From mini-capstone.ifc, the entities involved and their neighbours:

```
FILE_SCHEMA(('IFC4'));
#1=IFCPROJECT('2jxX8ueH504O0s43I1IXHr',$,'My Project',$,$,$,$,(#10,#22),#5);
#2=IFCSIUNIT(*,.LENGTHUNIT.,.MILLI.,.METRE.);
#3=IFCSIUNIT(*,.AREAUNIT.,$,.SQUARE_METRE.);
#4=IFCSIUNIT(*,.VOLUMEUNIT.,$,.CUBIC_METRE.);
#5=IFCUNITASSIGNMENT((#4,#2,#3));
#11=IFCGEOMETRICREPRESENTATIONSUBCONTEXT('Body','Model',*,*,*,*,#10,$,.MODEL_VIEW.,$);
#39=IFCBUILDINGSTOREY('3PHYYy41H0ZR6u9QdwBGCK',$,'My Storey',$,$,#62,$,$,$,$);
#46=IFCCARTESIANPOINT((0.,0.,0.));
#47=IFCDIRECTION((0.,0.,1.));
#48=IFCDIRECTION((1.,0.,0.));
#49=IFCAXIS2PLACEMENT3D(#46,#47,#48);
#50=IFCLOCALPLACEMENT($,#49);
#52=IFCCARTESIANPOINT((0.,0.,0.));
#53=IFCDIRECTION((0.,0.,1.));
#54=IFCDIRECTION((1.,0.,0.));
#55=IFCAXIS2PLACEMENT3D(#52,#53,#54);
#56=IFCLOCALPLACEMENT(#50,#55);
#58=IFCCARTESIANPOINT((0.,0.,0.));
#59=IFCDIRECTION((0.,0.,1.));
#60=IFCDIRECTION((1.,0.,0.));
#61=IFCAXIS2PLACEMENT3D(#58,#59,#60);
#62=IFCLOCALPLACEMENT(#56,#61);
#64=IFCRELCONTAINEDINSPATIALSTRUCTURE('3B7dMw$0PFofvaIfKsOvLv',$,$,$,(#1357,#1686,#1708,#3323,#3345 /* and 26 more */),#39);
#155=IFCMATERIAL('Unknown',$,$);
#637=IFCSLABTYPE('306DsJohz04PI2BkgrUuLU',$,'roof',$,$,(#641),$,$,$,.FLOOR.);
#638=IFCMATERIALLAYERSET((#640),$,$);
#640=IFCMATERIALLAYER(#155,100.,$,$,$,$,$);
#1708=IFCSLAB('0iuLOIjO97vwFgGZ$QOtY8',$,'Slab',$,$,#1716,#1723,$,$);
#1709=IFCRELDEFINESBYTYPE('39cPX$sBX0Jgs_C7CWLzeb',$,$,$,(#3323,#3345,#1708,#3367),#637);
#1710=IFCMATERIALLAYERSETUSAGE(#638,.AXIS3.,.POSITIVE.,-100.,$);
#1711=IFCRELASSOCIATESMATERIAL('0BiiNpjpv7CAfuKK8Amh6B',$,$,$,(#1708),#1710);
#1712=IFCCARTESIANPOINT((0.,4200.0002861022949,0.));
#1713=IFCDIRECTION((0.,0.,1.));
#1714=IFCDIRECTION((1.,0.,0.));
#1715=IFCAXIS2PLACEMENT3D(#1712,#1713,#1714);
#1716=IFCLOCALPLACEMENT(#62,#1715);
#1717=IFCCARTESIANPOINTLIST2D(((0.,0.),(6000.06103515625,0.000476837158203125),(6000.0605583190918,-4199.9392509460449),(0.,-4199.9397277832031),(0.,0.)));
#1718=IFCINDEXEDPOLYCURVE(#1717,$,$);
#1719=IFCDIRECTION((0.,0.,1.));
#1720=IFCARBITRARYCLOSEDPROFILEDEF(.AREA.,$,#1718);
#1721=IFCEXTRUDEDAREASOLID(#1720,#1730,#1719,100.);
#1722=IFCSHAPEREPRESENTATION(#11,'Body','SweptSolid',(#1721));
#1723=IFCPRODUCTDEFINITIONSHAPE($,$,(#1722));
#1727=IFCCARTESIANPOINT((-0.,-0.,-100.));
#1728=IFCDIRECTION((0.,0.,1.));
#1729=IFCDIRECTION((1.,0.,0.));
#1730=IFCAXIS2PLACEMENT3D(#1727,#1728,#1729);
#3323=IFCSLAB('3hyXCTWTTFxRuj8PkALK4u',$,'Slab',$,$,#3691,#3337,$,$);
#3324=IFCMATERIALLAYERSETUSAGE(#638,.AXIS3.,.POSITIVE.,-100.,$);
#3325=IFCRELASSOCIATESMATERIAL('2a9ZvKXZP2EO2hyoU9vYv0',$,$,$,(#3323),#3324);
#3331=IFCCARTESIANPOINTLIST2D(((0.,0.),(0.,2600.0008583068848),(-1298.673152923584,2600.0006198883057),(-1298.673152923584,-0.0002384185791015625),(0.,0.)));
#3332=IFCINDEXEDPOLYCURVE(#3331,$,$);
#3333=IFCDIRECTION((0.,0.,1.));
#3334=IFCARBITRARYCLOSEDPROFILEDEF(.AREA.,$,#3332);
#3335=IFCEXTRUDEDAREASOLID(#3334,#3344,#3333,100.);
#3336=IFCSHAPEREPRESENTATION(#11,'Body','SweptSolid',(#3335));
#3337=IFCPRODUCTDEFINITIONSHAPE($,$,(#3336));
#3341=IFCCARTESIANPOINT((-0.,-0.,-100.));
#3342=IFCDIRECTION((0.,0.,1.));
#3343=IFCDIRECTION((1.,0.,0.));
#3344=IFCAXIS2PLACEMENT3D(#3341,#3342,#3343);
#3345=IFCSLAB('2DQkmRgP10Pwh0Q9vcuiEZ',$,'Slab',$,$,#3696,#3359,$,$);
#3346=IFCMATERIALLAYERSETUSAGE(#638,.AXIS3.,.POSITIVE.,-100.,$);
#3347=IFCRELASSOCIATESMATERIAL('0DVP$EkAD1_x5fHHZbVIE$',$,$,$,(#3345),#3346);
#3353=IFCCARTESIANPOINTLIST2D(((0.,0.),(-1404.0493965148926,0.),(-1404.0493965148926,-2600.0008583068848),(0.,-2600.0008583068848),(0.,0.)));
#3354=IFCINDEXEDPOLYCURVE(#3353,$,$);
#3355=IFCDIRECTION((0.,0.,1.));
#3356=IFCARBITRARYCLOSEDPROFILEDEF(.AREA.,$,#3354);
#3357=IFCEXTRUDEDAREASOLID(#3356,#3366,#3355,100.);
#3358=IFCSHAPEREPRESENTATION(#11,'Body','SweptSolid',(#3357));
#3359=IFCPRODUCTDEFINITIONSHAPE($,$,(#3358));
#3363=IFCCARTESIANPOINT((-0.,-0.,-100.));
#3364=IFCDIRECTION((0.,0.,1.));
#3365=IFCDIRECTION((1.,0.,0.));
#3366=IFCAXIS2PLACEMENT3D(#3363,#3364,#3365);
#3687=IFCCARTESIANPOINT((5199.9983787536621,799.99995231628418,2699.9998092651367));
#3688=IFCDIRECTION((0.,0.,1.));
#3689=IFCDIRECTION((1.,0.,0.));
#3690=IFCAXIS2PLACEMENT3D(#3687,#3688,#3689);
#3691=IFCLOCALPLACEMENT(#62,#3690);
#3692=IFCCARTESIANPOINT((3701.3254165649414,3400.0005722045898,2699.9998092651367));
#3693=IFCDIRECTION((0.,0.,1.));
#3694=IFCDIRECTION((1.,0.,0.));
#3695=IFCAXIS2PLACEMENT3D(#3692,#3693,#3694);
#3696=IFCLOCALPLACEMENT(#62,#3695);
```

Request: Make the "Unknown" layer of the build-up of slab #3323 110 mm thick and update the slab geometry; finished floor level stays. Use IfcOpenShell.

```python
import ifcopenshell
import ifcopenshell.util.element
import ifcopenshell.util.representation

model = ifcopenshell.open("mini-capstone.ifc")

layer_set = model.by_id(638)
layer = next(l for l in layer_set.MaterialLayers if l.Material and l.Material.Name == "Unknown")
change = 110.0 - layer.LayerThickness
layer.LayerThickness += change

# The layer set is shared, so every slab that uses it gets the new thickness.
slabs = [e for e in ifcopenshell.util.element.get_elements_by_material(model, layer_set) if e.is_a("IfcSlab")]
for slab in sorted(slabs, key=lambda e: e.id()):
    body = ifcopenshell.util.representation.get_representation(slab, "Model", "Body")
    solid = body.Items[0]
    old_depth = solid.Depth
    solid.Depth += change
    # Extruded upwards: lower the start of the extrusion so the top stays.
    x, y, z = solid.Position.Location.Coordinates
    solid.Position.Location = model.createIfcCartesianPoint((x, y, z - change))
    print(slab.id(), f"{old_depth:g} -> {solid.Depth:g}")

# The layers are counted up from the underside, which has moved.
for usage in {ifcopenshell.util.element.get_material(slab) for slab in slabs}:
    usage.OffsetFromReferenceLine -= change

model.write("mini-capstone_updated.ifc")
```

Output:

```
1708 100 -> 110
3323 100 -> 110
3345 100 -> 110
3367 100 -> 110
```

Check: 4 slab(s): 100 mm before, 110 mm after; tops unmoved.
